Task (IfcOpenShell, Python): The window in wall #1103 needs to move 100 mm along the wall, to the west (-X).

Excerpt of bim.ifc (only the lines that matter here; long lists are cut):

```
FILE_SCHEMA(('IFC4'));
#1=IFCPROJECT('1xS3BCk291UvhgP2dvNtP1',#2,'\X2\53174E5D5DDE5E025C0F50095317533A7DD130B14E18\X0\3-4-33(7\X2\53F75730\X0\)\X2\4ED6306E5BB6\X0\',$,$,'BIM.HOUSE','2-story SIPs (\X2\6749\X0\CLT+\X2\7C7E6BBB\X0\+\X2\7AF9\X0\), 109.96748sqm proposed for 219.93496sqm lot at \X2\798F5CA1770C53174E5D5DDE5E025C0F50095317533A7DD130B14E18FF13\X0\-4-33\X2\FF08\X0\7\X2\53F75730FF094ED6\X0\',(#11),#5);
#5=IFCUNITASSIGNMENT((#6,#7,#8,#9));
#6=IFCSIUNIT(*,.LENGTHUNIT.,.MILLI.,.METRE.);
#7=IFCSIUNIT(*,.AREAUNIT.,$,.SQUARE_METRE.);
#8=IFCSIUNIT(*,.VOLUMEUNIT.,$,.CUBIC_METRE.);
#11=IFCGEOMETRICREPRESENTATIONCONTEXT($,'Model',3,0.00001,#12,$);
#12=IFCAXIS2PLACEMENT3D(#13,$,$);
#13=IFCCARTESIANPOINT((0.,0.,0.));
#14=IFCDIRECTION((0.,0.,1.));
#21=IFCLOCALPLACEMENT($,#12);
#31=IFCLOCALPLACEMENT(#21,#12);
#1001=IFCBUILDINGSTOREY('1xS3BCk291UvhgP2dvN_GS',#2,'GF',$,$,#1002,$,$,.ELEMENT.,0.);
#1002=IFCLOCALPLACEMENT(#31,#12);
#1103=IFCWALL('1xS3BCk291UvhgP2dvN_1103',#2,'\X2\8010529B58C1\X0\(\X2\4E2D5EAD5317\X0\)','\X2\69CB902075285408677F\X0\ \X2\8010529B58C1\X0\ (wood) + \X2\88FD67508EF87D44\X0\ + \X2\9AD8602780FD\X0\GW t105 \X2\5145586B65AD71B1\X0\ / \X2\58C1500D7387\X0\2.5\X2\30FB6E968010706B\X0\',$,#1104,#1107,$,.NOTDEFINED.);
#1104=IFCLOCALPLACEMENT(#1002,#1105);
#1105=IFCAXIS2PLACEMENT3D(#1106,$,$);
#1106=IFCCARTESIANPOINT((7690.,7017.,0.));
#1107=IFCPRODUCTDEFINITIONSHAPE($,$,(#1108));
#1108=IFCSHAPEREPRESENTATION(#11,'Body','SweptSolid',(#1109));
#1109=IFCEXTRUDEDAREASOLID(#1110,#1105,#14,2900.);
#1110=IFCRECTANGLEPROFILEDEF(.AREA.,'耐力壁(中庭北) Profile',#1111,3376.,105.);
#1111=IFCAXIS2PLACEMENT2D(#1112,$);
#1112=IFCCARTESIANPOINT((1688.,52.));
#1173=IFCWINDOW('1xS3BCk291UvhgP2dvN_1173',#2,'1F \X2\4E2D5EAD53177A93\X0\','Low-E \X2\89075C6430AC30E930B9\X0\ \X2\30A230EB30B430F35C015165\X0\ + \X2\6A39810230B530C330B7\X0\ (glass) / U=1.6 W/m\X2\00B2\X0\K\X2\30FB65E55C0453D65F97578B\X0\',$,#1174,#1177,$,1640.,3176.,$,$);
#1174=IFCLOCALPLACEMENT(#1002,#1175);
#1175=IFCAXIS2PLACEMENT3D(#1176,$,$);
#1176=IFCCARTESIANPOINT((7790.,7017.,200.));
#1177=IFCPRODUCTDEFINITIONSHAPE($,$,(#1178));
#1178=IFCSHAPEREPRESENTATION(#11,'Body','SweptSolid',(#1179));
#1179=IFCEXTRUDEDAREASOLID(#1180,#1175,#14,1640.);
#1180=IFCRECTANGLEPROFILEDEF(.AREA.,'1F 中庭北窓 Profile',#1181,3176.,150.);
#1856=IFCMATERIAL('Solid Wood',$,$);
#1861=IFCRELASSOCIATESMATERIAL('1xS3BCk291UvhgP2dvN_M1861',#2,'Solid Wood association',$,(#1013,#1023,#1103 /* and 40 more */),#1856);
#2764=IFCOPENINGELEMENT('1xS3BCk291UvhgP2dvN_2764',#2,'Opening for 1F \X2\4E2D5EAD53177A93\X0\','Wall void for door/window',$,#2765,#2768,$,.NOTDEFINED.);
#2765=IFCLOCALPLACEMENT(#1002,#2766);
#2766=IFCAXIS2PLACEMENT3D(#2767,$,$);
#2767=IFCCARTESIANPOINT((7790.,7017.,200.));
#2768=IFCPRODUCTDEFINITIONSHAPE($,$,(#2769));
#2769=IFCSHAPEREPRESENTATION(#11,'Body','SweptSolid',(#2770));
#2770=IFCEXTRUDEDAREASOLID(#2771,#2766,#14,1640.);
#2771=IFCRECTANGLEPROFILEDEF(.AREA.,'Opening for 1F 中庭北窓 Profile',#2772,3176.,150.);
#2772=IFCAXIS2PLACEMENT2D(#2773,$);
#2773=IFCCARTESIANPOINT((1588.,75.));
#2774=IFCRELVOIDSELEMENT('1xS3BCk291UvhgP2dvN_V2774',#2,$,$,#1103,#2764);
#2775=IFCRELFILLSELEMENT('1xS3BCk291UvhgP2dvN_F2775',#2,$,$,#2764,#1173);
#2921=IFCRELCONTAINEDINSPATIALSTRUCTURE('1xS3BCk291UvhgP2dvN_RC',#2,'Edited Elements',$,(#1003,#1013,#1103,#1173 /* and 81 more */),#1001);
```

```python
import ifcopenshell
import ifcopenshell.api.geometry
import ifcopenshell.util.placement
import ifcopenshell.util.unit

model = ifcopenshell.open("bim.ifc")
unit_scale = ifcopenshell.util.unit.calculate_unit_scale(model)

window = model.by_guid("1xS3BCk291UvhgP2dvN_1173")
opening = window.FillsVoids[0].RelatingOpeningElement
wall = opening.VoidsElements[0].RelatingBuildingElement

wall_matrix = ifcopenshell.util.placement.get_local_placement(wall.ObjectPlacement)
shift = wall_matrix[:3, 0] * -0.1 / unit_scale
before = ifcopenshell.util.placement.get_local_placement(window.ObjectPlacement)[:3, 3].copy()

# The window is not placed relative to its opening, so move both.
for product in (opening, window):
    matrix = ifcopenshell.util.placement.get_local_placement(product.ObjectPlacement)
    matrix[:3, 3] += shift
    ifcopenshell.api.geometry.edit_object_placement(model, product=product, matrix=matrix, is_si=False)

after = ifcopenshell.util.placement.get_local_placement(window.ObjectPlacement)[:3, 3]
print("window moved by", (after - before).round(3) + 0.0)

model.write("bim_updated.ifc")
```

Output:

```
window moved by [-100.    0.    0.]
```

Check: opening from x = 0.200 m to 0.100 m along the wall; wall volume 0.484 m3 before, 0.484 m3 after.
